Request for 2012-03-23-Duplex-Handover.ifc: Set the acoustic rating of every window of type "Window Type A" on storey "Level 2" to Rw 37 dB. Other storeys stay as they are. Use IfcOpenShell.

First a look at what the model holds.

```python
import ifcopenshell
import ifcopenshell.util.element

model = ifcopenshell.open("2012-03-23-Duplex-Handover.ifc")
print(model.schema)
storey = next(s for s in model.by_type("IfcBuildingStorey") if s.Name == "Level 2")
windows = [e for e in ifcopenshell.util.element.get_decomposition(storey) if e.is_a("IfcWindow")]
seen = {}
for e in windows:
    element_type = ifcopenshell.util.element.get_type(e)
    key = (element_type.Name if element_type != e and element_type else None, ifcopenshell.util.element.get_pset(e, "Pset_WindowCommon", "AcousticRating"))
    seen[key] = seen.get(key, 0) + 1
for (name, value), count in sorted(seen.items(), key=str):
    print(count, "x", name, "|", value)
```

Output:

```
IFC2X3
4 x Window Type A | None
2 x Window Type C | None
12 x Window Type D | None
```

```python
import ifcopenshell
import ifcopenshell.api.pset
import ifcopenshell.util.element

model = ifcopenshell.open("2012-03-23-Duplex-Handover.ifc")

storey = next(s for s in model.by_type("IfcBuildingStorey") if s.Name == "Level 2")
windows = [e for e in ifcopenshell.util.element.get_decomposition(storey) if e.is_a("IfcWindow")]

count = 0
for e in windows:
    element_type = ifcopenshell.util.element.get_type(e)
    if element_type in (None, e) or element_type.Name != "Window Type A":
        continue
    # add_pset returns the element's existing set when there is one.
    pset = ifcopenshell.api.pset.add_pset(model, product=e, name="Pset_WindowCommon")
    ifcopenshell.api.pset.edit_pset(model, pset=pset, properties={"AcousticRating": "Rw 37 dB"})
    count += 1

print(count, "windows updated")

model.write("2012-03-23-Duplex-Handover_edited.ifc")
```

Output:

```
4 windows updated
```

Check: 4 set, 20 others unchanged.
